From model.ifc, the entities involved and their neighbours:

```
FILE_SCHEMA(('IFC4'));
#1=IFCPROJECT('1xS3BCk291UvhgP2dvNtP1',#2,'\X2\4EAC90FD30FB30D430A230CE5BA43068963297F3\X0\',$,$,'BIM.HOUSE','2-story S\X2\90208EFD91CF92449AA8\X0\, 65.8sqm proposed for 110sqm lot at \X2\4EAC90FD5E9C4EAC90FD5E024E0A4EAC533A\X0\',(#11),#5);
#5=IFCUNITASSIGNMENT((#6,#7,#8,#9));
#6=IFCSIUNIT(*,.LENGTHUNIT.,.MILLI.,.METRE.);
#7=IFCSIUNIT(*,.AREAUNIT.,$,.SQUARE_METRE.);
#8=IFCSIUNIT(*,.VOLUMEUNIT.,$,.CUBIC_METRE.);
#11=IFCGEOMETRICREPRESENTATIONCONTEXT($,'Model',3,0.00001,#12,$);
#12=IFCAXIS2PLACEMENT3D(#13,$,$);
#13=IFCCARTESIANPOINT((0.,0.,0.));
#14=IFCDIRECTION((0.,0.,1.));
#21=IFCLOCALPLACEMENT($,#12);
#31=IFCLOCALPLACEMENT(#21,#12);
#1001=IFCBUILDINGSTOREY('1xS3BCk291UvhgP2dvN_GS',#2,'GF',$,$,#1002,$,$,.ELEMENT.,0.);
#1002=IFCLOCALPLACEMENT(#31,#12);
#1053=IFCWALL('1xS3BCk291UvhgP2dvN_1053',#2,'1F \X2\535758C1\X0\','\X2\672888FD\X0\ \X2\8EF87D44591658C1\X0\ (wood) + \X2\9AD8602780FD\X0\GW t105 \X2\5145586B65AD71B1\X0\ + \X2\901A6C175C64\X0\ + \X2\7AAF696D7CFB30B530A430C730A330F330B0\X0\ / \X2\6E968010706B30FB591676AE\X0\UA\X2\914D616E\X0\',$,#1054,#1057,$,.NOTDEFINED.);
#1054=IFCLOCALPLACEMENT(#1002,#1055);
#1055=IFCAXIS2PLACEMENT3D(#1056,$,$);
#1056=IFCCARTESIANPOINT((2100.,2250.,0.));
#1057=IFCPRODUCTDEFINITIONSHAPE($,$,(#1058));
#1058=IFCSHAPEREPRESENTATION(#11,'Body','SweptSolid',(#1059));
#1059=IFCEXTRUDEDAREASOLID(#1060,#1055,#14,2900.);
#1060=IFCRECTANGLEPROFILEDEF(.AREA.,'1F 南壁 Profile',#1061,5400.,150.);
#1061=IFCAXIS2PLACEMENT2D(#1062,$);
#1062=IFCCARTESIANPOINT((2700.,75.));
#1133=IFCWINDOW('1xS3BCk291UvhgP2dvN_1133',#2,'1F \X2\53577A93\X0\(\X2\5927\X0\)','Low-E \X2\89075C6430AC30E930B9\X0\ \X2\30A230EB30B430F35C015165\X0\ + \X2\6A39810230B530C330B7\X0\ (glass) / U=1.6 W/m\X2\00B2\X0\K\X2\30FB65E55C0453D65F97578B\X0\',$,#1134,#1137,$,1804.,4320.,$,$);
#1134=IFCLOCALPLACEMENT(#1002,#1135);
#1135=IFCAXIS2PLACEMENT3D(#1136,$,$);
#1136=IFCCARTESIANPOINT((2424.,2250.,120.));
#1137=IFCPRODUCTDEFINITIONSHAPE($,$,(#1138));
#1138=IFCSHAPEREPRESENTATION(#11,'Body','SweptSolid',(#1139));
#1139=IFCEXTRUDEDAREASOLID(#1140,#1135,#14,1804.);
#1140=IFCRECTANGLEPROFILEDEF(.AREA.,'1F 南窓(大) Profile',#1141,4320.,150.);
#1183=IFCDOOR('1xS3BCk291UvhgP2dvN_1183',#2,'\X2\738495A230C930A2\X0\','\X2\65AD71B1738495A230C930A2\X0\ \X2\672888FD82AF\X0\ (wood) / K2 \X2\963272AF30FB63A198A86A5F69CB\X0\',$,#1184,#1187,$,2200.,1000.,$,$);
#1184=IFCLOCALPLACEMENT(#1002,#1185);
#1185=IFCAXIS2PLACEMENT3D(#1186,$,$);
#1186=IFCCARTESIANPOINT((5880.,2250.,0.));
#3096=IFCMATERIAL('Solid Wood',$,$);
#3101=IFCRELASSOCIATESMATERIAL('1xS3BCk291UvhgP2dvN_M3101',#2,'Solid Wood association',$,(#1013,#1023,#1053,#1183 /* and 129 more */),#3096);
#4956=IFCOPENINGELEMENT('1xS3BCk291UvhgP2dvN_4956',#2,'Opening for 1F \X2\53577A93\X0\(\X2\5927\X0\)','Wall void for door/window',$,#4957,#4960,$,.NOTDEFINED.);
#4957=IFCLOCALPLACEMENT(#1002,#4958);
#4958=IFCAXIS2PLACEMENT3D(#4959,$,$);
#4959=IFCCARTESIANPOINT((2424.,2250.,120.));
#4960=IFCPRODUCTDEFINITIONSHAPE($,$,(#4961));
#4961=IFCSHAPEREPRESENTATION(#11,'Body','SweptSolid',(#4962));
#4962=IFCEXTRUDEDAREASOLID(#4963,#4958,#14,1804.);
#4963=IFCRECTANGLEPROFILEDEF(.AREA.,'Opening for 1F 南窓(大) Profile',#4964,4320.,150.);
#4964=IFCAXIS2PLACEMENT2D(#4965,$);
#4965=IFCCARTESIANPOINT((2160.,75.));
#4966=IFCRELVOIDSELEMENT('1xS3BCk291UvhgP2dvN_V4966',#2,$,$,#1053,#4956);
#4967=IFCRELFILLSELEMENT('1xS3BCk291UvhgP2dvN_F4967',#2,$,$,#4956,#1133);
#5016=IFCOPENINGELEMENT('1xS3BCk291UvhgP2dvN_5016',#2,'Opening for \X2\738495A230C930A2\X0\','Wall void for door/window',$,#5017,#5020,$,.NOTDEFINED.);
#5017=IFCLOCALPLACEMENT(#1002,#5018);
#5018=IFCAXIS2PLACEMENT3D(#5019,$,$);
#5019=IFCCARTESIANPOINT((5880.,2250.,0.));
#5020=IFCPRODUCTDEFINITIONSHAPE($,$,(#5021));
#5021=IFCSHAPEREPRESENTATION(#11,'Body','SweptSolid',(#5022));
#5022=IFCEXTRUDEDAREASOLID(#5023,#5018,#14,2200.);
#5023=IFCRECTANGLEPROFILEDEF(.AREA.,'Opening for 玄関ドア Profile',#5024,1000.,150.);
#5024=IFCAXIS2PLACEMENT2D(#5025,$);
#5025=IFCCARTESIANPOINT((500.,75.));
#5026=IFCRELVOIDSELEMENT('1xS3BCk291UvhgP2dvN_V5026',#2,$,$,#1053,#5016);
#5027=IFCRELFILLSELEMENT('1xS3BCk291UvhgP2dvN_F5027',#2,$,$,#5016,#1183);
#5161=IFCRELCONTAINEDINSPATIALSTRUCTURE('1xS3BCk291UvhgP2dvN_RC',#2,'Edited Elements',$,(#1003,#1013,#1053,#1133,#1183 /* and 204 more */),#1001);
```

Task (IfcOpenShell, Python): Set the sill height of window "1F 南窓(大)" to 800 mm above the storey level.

```python
import numpy as np
import ifcopenshell
import ifcopenshell.api.geometry
import ifcopenshell.geom
import ifcopenshell.util.element
import ifcopenshell.util.placement
import ifcopenshell.util.shape
import ifcopenshell.util.unit

model = ifcopenshell.open("model.ifc")
unit_scale = ifcopenshell.util.unit.calculate_unit_scale(model)

window = model.by_guid("1xS3BCk291UvhgP2dvN_1133")
opening = window.FillsVoids[0].RelatingOpeningElement
storey = ifcopenshell.util.element.get_container(window, ifc_class="IfcBuildingStorey")
level = ifcopenshell.util.placement.get_local_placement(storey.ObjectPlacement)[2, 3]

# The opening's origin need not be at the sill, so measure its lowest point.
shape = ifcopenshell.geom.create_shape(ifcopenshell.geom.settings(), opening)
bottom = ifcopenshell.util.shape.get_shape_bottom_elevation(shape, shape.geometry) / unit_scale
dz = level + 0.8 / unit_scale - bottom

shift = np.array([0.0, 0.0, dz])
# The window is not placed relative to its opening, so move both.
for product in (opening, window):
    matrix = ifcopenshell.util.placement.get_local_placement(product.ObjectPlacement)
    matrix[:3, 3] += shift
    ifcopenshell.api.geometry.edit_object_placement(model, product=product, matrix=matrix, is_si=False)

print(f"moved by {dz * unit_scale:+.3f} m")

model.write("model_v2.ifc")
```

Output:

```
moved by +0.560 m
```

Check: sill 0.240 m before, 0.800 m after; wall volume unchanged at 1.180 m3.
